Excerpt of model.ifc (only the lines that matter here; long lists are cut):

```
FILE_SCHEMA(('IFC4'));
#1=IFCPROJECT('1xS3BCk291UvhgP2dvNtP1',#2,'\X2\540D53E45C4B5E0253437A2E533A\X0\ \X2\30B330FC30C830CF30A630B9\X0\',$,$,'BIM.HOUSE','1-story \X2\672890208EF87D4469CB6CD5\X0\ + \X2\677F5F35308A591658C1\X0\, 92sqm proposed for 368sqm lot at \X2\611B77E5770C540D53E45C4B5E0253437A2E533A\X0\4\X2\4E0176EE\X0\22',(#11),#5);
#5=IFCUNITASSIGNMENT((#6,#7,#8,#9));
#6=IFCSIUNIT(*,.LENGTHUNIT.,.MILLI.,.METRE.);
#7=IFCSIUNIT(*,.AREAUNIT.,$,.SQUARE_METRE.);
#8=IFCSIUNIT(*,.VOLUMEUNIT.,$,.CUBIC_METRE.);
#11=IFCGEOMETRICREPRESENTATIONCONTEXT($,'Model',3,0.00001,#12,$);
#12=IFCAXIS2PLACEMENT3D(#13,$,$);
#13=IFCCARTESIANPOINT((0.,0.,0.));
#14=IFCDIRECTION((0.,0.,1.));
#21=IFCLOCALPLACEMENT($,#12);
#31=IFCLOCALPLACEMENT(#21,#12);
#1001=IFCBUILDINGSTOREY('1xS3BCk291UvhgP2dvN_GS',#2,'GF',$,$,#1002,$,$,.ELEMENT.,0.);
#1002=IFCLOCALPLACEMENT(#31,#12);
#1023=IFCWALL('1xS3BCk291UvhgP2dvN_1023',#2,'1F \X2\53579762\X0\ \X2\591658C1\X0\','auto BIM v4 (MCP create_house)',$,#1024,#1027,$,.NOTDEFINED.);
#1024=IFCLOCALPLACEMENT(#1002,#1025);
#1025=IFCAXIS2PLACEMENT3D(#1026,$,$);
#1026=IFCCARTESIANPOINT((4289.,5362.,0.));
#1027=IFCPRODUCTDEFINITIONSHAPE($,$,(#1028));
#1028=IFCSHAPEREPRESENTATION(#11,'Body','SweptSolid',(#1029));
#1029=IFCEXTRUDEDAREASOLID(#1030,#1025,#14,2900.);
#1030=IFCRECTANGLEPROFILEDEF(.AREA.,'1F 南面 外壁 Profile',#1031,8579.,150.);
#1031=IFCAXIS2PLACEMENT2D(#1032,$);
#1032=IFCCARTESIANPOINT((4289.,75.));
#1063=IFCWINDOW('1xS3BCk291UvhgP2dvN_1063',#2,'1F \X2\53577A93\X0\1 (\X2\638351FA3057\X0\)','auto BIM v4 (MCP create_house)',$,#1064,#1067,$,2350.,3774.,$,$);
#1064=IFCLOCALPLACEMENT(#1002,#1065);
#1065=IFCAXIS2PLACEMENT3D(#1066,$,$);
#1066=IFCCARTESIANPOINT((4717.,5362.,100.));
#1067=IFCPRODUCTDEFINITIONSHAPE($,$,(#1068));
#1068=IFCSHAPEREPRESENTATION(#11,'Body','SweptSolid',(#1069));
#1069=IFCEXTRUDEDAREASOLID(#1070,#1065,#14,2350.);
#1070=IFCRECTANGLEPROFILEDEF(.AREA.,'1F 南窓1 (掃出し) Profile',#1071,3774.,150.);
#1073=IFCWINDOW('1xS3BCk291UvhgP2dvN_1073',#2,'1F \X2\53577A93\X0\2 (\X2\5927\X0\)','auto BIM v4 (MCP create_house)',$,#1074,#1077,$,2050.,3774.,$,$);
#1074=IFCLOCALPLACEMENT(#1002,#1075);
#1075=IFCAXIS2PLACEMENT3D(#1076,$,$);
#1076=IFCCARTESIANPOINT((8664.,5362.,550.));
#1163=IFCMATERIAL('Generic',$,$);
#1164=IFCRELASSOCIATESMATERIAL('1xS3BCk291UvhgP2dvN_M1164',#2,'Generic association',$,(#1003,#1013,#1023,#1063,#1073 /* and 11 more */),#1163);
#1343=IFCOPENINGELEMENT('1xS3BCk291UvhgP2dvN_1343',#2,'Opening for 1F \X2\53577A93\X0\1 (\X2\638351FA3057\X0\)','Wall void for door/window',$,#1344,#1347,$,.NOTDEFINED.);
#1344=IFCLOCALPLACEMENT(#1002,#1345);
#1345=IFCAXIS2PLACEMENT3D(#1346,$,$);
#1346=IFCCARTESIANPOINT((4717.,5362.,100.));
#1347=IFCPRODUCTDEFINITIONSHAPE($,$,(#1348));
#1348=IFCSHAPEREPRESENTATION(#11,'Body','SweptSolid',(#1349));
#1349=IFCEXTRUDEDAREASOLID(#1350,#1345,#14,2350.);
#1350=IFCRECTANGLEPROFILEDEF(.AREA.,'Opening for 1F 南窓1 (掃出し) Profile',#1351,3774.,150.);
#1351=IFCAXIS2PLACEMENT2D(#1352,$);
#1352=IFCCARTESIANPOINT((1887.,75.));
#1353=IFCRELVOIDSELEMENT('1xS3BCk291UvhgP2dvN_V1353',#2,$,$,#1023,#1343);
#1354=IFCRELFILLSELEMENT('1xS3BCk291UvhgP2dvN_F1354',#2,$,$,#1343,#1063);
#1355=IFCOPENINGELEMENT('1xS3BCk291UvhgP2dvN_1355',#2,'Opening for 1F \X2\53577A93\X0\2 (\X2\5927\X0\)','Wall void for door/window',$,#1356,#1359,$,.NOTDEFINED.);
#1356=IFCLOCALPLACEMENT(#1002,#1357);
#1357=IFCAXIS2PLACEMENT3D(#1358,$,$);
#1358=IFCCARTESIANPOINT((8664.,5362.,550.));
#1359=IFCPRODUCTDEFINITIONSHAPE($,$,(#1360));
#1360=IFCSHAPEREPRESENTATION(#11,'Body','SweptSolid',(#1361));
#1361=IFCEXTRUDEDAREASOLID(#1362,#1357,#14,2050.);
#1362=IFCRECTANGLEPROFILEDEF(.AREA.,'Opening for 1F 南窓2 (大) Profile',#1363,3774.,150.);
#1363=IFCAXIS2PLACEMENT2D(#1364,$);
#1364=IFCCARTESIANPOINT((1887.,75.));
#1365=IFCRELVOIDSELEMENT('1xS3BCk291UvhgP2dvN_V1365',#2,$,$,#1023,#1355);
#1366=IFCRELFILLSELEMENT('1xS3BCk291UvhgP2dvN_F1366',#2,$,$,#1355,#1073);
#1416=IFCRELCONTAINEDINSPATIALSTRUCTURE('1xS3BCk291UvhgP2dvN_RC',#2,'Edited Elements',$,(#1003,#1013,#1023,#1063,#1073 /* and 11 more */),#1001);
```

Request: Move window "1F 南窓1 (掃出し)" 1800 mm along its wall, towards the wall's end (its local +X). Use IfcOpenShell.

```python
import ifcopenshell
import ifcopenshell.api.geometry
import ifcopenshell.util.placement
import ifcopenshell.util.unit

model = ifcopenshell.open("model.ifc")
unit_scale = ifcopenshell.util.unit.calculate_unit_scale(model)

window = model.by_guid("1xS3BCk291UvhgP2dvN_1063")
opening = window.FillsVoids[0].RelatingOpeningElement
wall = opening.VoidsElements[0].RelatingBuildingElement

wall_matrix = ifcopenshell.util.placement.get_local_placement(wall.ObjectPlacement)
shift = wall_matrix[:3, 0] * 1.8 / unit_scale
before = ifcopenshell.util.placement.get_local_placement(window.ObjectPlacement)[:3, 3].copy()

# The window is not placed relative to its opening, so move both.
for product in (opening, window):
    matrix = ifcopenshell.util.placement.get_local_placement(product.ObjectPlacement)
    matrix[:3, 3] += shift
    ifcopenshell.api.geometry.edit_object_placement(model, product=product, matrix=matrix, is_si=False)

after = ifcopenshell.util.placement.get_local_placement(window.ObjectPlacement)[:3, 3]
print("window moved by", (after - before).round(3) + 0.0)

model.write("model_updated.ifc")
```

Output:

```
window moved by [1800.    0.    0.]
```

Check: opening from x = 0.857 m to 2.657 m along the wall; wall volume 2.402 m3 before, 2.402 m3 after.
